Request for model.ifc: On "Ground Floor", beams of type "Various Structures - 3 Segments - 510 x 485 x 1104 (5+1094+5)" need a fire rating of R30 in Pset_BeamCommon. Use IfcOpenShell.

First a look at what the model holds.

```python
import ifcopenshell
import ifcopenshell.util.element

model = ifcopenshell.open("model.ifc")
print(model.schema)
storey = next(s for s in model.by_type("IfcBuildingStorey") if s.Name == "Ground Floor")
beams = [e for e in ifcopenshell.util.element.get_decomposition(storey) if e.is_a("IfcBeam")]
seen = {}
for e in beams:
    element_type = ifcopenshell.util.element.get_type(e)
    key = (element_type.Name if element_type != e and element_type else None, ifcopenshell.util.element.get_pset(e, "Pset_BeamCommon", "FireRating"))
    seen[key] = seen.get(key, 0) + 1
for (name, value), count in sorted(seen.items(), key=str):
    print(count, "x", name, "|", value)
```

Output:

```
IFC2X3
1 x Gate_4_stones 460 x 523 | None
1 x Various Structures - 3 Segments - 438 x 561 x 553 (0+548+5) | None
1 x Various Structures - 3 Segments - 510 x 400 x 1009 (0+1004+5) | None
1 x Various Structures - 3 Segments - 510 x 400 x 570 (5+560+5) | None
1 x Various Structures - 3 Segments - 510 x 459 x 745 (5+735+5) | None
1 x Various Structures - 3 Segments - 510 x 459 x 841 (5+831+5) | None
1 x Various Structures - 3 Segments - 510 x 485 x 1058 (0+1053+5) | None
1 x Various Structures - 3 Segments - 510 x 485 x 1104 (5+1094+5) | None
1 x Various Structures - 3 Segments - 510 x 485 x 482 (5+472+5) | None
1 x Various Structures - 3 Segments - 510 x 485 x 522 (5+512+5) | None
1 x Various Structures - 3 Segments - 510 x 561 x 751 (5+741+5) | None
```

```python
import ifcopenshell
import ifcopenshell.api.pset
import ifcopenshell.util.element

model = ifcopenshell.open("model.ifc")

storey = next(s for s in model.by_type("IfcBuildingStorey") if s.Name == "Ground Floor")
beams = [e for e in ifcopenshell.util.element.get_decomposition(storey) if e.is_a("IfcBeam")]

count = 0
for e in beams:
    element_type = ifcopenshell.util.element.get_type(e)
    if element_type in (None, e) or element_type.Name != "Various Structures - 3 Segments - 510 x 485 x 1104 (5+1094+5)":
        continue
    # add_pset returns the element's existing set when there is one.
    pset = ifcopenshell.api.pset.add_pset(model, product=e, name="Pset_BeamCommon")
    ifcopenshell.api.pset.edit_pset(model, pset=pset, properties={"FireRating": "R30"})
    count += 1

print(count, "beams updated")

model.write("model_rev.ifc")
```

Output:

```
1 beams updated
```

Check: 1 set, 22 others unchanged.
